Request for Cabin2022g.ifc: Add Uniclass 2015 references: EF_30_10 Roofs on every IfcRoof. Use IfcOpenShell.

First a look at what the model holds.

```python
import ifcopenshell

model = ifcopenshell.open("Cabin2022g.ifc")
print(model.schema)
print("classifications:", [c.Name for c in model.by_type("IfcClassification")])
for ifc_class in ("IfcDoor", "IfcRoof", "IfcStair", "IfcWall", "IfcWindow"):
    print(ifc_class, len(model.by_type(ifc_class)))
```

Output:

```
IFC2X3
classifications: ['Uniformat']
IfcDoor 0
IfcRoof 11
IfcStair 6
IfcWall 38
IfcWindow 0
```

```python
import ifcopenshell
import ifcopenshell.api.classification

model = ifcopenshell.open("Cabin2022g.ifc")

# IFC2X3 requires Source and Edition and has no link from the project to the system.
system = model.create_entity("IfcClassification", Source="NBS", Edition="2015", Name="Uniclass 2015")

codes = {
    "IfcRoof": ("EF_30_10", "Roofs"),
}
for ifc_class, (code, name) in codes.items():
    products = model.by_type(ifc_class)
    ifcopenshell.api.classification.add_reference(
        model, products=products, classification=system, identification=code, name=name
    )
    print(code, len(products))

model.write("Cabin2022g_rev.ifc")
```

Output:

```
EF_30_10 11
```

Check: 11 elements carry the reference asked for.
